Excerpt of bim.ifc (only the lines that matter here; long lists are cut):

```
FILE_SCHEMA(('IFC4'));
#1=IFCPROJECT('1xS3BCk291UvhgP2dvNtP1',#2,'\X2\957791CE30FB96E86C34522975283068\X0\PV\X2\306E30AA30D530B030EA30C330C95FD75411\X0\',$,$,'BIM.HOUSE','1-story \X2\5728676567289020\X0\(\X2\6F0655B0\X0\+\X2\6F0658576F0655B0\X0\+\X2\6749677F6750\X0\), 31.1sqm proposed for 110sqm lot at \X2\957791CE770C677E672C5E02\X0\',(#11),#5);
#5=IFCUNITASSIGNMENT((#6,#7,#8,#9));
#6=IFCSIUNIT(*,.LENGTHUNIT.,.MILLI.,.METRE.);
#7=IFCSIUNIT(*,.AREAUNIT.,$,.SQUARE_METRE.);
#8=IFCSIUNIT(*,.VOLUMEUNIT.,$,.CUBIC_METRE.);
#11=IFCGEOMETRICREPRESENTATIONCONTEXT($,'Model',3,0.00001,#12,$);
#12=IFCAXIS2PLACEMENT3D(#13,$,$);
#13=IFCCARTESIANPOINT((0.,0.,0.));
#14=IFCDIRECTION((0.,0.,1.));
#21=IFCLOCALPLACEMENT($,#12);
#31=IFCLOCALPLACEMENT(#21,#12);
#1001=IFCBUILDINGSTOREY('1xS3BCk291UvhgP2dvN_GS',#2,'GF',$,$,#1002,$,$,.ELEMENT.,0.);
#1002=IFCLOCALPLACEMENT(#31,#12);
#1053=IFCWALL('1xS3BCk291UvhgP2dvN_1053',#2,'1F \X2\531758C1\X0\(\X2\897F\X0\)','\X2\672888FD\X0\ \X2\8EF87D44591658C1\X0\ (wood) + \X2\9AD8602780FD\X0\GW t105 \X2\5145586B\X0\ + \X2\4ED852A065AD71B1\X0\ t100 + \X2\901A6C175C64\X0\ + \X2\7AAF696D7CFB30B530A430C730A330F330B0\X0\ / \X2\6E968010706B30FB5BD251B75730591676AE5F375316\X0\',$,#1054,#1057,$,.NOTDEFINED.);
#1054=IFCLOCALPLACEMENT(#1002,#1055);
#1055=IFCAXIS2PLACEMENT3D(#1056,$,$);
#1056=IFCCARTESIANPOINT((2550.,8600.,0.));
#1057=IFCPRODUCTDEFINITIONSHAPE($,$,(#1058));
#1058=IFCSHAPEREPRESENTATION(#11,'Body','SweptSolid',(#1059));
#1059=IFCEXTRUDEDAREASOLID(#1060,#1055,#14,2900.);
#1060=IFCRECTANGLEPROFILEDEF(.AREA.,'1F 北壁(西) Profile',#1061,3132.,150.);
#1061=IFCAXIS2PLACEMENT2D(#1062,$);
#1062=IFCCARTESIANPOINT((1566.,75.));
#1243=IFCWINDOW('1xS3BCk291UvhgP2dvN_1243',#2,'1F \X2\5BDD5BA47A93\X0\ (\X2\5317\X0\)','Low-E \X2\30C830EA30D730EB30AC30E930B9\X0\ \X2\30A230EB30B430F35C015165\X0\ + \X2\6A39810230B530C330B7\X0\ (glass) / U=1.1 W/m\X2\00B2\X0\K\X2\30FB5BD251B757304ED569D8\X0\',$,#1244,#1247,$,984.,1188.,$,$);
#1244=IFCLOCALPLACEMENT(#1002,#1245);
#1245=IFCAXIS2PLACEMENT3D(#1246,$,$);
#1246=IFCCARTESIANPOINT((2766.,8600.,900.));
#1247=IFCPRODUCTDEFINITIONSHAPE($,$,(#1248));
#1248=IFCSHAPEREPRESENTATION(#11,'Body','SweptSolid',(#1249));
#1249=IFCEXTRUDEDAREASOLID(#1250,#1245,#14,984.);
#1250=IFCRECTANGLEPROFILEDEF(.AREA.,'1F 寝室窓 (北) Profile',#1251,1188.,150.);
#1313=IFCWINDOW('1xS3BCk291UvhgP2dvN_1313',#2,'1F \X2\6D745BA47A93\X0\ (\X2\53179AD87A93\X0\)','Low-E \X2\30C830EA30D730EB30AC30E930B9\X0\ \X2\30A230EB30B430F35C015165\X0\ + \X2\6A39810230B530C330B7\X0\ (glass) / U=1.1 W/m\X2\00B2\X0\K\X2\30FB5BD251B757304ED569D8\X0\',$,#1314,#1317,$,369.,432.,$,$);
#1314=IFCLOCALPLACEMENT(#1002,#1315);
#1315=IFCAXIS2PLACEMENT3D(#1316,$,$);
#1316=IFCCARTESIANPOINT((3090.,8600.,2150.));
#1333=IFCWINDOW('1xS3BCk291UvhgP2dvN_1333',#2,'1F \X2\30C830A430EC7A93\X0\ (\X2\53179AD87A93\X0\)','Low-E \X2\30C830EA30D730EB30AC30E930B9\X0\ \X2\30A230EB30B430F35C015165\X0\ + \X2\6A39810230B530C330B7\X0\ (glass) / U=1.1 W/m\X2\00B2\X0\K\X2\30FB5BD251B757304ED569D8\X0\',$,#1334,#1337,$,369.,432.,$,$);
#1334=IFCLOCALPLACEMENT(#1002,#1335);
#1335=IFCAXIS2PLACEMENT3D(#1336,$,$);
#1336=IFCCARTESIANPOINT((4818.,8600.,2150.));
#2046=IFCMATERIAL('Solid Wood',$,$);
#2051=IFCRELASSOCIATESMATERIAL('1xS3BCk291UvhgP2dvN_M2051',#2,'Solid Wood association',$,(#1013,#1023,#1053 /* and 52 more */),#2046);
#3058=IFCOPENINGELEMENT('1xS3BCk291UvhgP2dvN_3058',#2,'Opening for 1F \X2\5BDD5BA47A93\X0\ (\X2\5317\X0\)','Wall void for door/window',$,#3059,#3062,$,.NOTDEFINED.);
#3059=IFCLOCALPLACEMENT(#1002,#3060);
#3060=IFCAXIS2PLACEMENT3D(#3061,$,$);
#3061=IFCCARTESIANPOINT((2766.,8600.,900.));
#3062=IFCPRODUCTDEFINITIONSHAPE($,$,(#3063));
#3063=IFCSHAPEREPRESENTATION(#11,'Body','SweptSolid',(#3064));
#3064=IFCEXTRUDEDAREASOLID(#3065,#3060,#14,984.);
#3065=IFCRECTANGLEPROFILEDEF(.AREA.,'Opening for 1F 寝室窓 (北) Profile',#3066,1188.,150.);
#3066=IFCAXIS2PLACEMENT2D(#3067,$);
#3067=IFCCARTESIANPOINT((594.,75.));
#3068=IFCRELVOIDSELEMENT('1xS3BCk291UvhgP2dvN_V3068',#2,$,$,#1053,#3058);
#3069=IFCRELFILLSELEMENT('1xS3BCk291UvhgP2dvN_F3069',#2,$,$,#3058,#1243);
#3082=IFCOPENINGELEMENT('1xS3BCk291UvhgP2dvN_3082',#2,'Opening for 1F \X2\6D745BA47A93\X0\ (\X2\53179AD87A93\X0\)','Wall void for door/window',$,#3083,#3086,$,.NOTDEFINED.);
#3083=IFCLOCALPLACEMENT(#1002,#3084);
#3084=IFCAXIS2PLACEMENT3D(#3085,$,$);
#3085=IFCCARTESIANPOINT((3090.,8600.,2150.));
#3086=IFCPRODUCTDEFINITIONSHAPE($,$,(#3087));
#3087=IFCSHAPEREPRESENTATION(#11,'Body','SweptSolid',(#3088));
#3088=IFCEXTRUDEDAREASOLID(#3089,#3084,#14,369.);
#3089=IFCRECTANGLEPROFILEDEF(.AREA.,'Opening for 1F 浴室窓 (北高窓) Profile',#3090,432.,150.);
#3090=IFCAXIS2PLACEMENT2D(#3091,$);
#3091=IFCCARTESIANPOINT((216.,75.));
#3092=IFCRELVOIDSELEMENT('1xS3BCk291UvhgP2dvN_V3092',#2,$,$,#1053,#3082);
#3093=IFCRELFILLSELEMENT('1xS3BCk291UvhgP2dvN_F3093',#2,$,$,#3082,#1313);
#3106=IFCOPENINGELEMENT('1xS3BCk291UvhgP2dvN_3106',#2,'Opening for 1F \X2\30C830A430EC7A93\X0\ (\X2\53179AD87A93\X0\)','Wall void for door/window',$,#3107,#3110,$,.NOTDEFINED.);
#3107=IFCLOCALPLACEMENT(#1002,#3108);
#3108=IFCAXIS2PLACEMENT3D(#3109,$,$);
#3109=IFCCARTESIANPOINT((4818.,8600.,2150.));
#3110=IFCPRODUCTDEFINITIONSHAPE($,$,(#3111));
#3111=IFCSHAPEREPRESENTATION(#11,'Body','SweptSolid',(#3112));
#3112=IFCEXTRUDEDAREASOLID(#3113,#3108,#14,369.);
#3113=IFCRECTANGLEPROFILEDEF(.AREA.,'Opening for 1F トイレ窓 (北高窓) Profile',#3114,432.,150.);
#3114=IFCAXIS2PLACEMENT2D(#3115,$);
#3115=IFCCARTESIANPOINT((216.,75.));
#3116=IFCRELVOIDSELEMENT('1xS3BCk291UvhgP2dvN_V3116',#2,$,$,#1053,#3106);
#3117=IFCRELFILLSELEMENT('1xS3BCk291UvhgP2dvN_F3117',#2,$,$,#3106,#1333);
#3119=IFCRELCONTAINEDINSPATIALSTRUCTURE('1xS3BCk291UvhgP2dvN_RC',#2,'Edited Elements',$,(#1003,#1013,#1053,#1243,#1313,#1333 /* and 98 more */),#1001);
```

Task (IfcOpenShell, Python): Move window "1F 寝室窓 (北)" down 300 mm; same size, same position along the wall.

```python
import numpy as np
import ifcopenshell
import ifcopenshell.api.geometry
import ifcopenshell.util.placement
import ifcopenshell.util.unit

model = ifcopenshell.open("bim.ifc")
unit_scale = ifcopenshell.util.unit.calculate_unit_scale(model)

window = model.by_guid("1xS3BCk291UvhgP2dvN_1243")
opening = window.FillsVoids[0].RelatingOpeningElement
dz = -0.3 / unit_scale

shift = np.array([0.0, 0.0, dz])
# The window is not placed relative to its opening, so move both.
for product in (opening, window):
    matrix = ifcopenshell.util.placement.get_local_placement(product.ObjectPlacement)
    matrix[:3, 3] += shift
    ifcopenshell.api.geometry.edit_object_placement(model, product=product, matrix=matrix, is_si=False)

print(f"moved by {dz * unit_scale:+.3f} m")

model.write("bim_rev.ifc")
```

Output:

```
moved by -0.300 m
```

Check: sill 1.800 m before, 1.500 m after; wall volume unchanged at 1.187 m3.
